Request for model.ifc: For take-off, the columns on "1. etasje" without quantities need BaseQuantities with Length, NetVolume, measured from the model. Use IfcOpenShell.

First a look at what the model holds.

```python
import ifcopenshell
import ifcopenshell.util.element
import ifcopenshell.util.unit

model = ifcopenshell.open("model.ifc")
print(model.schema)
for unit_type in ("LENGTHUNIT", "AREAUNIT", "VOLUMEUNIT"):
    print(unit_type, ifcopenshell.util.unit.calculate_unit_scale(model, unit_type))
storey = next(s for s in model.by_type("IfcBuildingStorey") if s.Name == "1. etasje")
columns = [e for e in ifcopenshell.util.element.get_decomposition(storey) if e.is_a("IfcColumn")]
for e in sorted(columns, key=lambda e: e.id()):
    print(e.id(), e.is_a(), e.Name, list(ifcopenshell.util.element.get_psets(e, qtos_only=True)), sep=" | ")
```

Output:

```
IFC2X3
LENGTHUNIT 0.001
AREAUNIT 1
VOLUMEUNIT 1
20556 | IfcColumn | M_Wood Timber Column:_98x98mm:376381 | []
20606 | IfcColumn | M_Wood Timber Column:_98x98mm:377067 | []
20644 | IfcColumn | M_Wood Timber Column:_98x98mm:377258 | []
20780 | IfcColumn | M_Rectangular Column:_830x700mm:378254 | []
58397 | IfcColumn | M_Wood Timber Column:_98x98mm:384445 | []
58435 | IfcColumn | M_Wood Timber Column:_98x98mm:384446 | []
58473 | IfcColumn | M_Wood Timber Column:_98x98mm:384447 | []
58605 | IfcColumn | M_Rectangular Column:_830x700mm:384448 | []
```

```python
import ifcopenshell
import ifcopenshell.api.pset
import ifcopenshell.geom
import ifcopenshell.util.element
import ifcopenshell.util.shape
import ifcopenshell.util.unit

model = ifcopenshell.open("model.ifc")
unit_scale = ifcopenshell.util.unit.calculate_unit_scale(model)
volume_scale = ifcopenshell.util.unit.calculate_unit_scale(model, "VOLUMEUNIT")
settings = ifcopenshell.geom.settings()

storey = next(s for s in model.by_type("IfcBuildingStorey") if s.Name == "1. etasje")
columns = [e for e in ifcopenshell.util.element.get_decomposition(storey) if e.is_a("IfcColumn")]

for e in sorted(columns, key=lambda e: e.id()):
    if ifcopenshell.util.element.get_psets(e, qtos_only=True, should_inherit=False):
        continue
    # Geometry comes back in metres, in the element's own axes.
    shape = ifcopenshell.geom.create_shape(settings, e)
    values = {
        "Length": ifcopenshell.util.shape.get_z(shape.geometry) / unit_scale,
        "NetVolume": ifcopenshell.util.shape.get_volume(shape.geometry) / volume_scale,
    }
    qto = ifcopenshell.api.pset.add_qto(model, product=e, name="BaseQuantities")
    ifcopenshell.api.pset.edit_qto(model, qto=qto, properties=values)
    print(e.id(), {k: round(v, 3) for k, v in values.items()})

model.write("model_rev.ifc")
```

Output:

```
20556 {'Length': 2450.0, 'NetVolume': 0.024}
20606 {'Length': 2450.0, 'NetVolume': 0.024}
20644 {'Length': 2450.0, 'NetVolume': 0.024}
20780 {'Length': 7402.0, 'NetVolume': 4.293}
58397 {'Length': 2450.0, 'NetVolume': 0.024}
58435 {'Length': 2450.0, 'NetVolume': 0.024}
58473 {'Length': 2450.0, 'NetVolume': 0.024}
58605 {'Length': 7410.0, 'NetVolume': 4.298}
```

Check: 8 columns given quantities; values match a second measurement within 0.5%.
